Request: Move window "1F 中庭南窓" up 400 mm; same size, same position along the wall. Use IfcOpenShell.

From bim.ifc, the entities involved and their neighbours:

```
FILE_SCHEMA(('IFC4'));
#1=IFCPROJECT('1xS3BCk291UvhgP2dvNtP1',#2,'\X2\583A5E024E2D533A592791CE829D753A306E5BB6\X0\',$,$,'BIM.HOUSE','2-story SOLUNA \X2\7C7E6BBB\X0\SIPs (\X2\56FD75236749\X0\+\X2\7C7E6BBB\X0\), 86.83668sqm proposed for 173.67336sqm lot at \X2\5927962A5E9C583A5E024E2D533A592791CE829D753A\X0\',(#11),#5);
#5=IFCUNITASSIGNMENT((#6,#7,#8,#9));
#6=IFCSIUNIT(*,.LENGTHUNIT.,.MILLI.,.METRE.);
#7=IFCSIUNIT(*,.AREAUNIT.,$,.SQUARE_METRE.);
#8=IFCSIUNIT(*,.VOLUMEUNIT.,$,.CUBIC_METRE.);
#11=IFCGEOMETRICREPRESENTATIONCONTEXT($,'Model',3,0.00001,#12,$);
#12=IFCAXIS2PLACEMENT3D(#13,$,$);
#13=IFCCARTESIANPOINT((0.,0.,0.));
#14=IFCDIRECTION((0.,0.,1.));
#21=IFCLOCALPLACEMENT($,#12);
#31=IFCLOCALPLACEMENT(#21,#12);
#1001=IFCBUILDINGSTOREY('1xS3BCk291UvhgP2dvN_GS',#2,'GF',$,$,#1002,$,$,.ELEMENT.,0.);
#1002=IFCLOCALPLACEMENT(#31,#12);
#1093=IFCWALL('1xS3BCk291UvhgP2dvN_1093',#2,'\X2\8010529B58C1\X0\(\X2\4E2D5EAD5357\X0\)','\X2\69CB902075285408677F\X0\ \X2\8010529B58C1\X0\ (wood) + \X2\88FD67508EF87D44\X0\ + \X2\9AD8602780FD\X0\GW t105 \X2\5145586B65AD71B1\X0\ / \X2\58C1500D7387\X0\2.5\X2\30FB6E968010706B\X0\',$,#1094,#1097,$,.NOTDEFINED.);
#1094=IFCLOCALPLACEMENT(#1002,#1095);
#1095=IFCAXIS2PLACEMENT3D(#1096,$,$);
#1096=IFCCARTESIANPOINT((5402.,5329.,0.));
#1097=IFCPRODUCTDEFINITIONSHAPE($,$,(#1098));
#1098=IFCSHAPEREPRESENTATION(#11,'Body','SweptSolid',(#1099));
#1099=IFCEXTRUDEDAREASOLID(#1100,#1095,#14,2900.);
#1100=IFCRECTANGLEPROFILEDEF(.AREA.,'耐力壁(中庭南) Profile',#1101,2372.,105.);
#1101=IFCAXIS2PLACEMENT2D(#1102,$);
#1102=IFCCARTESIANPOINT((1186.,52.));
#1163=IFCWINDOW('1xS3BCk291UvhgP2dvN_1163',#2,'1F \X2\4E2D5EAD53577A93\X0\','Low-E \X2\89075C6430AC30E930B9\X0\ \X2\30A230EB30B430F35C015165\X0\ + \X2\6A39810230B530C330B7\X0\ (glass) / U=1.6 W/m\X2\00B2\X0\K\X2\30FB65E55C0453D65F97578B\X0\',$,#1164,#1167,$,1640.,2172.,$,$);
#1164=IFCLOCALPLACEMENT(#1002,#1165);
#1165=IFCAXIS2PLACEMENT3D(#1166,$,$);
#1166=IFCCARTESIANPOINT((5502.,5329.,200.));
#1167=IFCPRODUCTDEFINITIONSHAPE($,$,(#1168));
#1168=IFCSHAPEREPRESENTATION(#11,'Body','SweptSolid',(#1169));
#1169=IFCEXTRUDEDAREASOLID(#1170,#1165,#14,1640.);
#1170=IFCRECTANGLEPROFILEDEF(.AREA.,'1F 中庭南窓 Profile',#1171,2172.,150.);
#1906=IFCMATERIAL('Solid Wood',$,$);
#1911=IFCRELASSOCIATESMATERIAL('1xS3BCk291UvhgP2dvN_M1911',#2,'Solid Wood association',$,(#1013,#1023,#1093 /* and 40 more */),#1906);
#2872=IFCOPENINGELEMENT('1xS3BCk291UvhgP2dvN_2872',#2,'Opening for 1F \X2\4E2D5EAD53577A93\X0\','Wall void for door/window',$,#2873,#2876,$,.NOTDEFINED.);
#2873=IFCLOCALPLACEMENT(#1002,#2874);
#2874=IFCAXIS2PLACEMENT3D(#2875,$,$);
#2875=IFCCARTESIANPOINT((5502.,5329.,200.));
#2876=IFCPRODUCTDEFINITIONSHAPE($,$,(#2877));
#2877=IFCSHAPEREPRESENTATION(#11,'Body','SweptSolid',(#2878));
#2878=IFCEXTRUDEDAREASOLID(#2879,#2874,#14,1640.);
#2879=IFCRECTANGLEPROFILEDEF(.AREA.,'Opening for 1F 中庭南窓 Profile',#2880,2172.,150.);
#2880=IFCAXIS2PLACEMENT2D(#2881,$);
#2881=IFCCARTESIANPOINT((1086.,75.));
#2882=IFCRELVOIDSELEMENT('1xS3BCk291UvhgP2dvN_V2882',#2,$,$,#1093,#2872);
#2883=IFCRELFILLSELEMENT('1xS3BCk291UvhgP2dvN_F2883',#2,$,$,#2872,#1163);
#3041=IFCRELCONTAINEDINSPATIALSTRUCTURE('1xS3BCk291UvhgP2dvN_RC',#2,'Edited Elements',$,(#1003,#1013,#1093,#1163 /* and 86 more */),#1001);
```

```python
import numpy as np
import ifcopenshell
import ifcopenshell.api.geometry
import ifcopenshell.util.placement
import ifcopenshell.util.unit

model = ifcopenshell.open("bim.ifc")
unit_scale = ifcopenshell.util.unit.calculate_unit_scale(model)

window = model.by_id(1163)
opening = window.FillsVoids[0].RelatingOpeningElement
dz = 400.0

shift = np.array([0.0, 0.0, dz])
# The window is not placed relative to its opening, so move both.
for product in (opening, window):
    matrix = ifcopenshell.util.placement.get_local_placement(product.ObjectPlacement)
    matrix[:3, 3] += shift
    ifcopenshell.api.geometry.edit_object_placement(model, product=product, matrix=matrix, is_si=False)

print(f"moved by {dz * unit_scale:+.3f} m")

model.write("bim_edited.ifc")
```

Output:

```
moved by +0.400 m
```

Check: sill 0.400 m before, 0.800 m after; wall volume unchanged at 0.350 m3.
